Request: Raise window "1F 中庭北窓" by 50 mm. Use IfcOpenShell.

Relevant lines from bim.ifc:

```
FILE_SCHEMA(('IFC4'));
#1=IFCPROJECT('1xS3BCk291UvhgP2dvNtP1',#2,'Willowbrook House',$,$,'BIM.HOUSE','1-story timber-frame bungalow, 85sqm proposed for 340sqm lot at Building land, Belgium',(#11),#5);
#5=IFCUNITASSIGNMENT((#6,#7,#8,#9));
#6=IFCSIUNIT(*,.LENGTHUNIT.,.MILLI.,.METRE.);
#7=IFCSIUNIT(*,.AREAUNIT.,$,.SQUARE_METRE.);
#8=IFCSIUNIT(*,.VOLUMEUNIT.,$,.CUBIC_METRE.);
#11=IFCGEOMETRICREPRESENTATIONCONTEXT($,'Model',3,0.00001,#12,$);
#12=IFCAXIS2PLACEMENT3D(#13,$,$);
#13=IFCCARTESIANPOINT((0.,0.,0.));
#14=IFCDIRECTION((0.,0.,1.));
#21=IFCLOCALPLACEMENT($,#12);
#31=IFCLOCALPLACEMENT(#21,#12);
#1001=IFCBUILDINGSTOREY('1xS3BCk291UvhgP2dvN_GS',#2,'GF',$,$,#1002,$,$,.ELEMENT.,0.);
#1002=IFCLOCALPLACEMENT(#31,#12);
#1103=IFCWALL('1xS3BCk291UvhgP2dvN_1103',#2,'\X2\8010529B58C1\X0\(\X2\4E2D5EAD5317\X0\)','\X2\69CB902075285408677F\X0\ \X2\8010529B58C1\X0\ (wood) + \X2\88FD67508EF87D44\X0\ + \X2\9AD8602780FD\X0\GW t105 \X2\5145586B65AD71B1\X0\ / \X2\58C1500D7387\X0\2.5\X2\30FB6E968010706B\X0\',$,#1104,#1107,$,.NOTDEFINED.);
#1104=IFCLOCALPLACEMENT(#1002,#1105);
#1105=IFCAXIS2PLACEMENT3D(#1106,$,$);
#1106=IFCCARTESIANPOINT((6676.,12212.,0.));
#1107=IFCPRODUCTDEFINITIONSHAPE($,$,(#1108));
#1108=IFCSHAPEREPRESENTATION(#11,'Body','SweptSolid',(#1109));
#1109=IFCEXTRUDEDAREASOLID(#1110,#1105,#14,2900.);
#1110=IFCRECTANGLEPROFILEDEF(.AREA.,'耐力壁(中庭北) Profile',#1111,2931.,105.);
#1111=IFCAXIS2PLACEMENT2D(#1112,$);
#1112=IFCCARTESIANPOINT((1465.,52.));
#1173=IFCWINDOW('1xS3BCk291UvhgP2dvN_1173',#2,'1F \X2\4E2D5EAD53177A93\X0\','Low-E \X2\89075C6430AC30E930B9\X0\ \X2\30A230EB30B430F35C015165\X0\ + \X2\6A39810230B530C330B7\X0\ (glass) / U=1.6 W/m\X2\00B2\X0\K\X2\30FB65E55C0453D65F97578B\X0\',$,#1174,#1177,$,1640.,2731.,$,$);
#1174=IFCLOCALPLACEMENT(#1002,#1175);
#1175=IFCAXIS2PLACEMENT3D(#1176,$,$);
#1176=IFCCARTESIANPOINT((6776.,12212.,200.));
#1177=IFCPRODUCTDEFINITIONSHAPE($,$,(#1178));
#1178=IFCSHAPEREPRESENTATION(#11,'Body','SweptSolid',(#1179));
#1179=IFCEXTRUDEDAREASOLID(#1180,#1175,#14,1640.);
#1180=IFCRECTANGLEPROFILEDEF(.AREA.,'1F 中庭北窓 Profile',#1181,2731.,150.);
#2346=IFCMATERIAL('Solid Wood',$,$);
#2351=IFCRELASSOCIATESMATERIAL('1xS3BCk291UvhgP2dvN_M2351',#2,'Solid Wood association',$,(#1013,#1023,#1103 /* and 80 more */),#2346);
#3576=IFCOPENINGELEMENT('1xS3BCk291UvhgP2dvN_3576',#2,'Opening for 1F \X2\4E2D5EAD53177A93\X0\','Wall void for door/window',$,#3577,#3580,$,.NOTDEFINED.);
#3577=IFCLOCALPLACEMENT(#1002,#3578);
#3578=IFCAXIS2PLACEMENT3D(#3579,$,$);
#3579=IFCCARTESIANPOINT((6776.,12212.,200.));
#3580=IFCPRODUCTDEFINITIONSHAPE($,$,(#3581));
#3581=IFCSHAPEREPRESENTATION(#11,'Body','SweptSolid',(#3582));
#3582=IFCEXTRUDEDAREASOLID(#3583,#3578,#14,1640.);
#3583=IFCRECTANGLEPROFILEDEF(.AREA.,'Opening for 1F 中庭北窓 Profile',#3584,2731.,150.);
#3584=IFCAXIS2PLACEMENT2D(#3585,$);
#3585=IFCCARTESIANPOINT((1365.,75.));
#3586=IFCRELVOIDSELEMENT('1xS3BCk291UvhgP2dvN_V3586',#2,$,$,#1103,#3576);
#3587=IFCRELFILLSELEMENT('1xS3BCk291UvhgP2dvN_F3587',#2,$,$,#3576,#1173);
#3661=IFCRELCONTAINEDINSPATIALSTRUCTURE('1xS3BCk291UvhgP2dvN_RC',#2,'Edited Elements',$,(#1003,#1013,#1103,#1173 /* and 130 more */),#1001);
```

```python
import numpy as np
import ifcopenshell
import ifcopenshell.api.geometry
import ifcopenshell.util.placement
import ifcopenshell.util.unit

model = ifcopenshell.open("bim.ifc")
unit_scale = ifcopenshell.util.unit.calculate_unit_scale(model)

window = model.by_id(1173)
opening = window.FillsVoids[0].RelatingOpeningElement
dz = 0.05 / unit_scale

shift = np.array([0.0, 0.0, dz])
# The window is not placed relative to its opening, so move both.
for product in (opening, window):
    matrix = ifcopenshell.util.placement.get_local_placement(product.ObjectPlacement)
    matrix[:3, 3] += shift
    ifcopenshell.api.geometry.edit_object_placement(model, product=product, matrix=matrix, is_si=False)

print(f"moved by {dz * unit_scale:+.3f} m")

model.write("bim_v2.ifc")
```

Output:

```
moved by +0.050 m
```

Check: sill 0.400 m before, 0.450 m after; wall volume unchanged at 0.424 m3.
